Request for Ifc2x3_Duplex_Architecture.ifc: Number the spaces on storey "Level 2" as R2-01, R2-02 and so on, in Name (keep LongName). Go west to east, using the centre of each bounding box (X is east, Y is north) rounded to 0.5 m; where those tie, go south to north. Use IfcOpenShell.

First a look at what the model holds.

```python
import ifcopenshell
import ifcopenshell.util.element
import ifcopenshell.util.placement

model = ifcopenshell.open("Ifc2x3_Duplex_Architecture.ifc")
print(model.schema)
storey = next(s for s in model.by_type("IfcBuildingStorey") if s.Name == "Level 2")
spaces = [e for e in ifcopenshell.util.element.get_decomposition(storey) if e.is_a("IfcSpace")]
for e in sorted(spaces, key=lambda e: e.id()):
    origin = ifcopenshell.util.placement.get_local_placement(e.ObjectPlacement)[:3, 3]
    print(e.id(), e.Name, e.LongName, origin.round(2) + 0.0, sep=" | ")
```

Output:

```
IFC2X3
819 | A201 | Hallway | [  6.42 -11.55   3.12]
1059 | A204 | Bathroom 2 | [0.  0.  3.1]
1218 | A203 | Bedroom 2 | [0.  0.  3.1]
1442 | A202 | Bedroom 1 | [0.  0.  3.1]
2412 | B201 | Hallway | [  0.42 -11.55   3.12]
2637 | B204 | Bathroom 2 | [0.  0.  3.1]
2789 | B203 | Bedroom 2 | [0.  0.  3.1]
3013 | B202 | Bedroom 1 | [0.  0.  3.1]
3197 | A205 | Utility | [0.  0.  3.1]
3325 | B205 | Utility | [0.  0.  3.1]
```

```python
import ifcopenshell
import ifcopenshell.geom
import ifcopenshell.util.element
import ifcopenshell.util.shape

model = ifcopenshell.open("Ifc2x3_Duplex_Architecture.ifc")
settings = ifcopenshell.geom.settings()
settings.set("use-world-coords", True)


def centre(element):
    shape = ifcopenshell.geom.create_shape(settings, element)
    return ifcopenshell.util.shape.get_bbox_centroid(shape.geometry)


storey = next(s for s in model.by_type("IfcBuildingStorey") if s.Name == "Level 2")
spaces = [e for e in ifcopenshell.util.element.get_decomposition(storey) if e.is_a("IfcSpace")]

# Insertion points can sit at a corner or the storey origin, so sort by the geometry (in metres).
centres = {e: centre(e) for e in spaces}
spaces.sort(key=lambda e: (round(centres[e][0] / 0.5), centres[e][1]))

for i, e in enumerate(spaces, start=1):
    number = f"R2-{i:02d}"
    e.Name = number
    print(e.id(), number)

model.write("Ifc2x3_Duplex_Architecture_updated.ifc")
```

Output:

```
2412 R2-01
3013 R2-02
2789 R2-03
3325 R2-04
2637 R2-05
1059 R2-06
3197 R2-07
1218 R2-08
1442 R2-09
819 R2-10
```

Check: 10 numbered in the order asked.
